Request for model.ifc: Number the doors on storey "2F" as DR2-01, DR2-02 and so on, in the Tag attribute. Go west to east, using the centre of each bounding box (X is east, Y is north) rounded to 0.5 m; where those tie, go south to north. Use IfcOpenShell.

First a look at what the model holds.

```python
import ifcopenshell
import ifcopenshell.util.element
import ifcopenshell.util.placement

model = ifcopenshell.open("model.ifc")
print(model.schema)
storey = next(s for s in model.by_type("IfcBuildingStorey") if s.Name == "2F")
doors = [e for e in ifcopenshell.util.element.get_decomposition(storey) if e.is_a("IfcDoor")]
for e in sorted(doors, key=lambda e: e.id()):
    origin = ifcopenshell.util.placement.get_local_placement(e.ObjectPlacement)[:3, 3]
    print(e.id(), e.Tag, e.Name, origin.round(2) + 0.0, sep=" | ")
```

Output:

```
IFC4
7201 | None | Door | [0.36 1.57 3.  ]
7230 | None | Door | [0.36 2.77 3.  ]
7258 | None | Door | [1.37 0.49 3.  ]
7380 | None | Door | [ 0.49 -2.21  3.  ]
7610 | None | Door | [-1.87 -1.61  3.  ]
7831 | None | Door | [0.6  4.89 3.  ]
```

```python
import ifcopenshell
import ifcopenshell.geom
import ifcopenshell.util.element
import ifcopenshell.util.shape

model = ifcopenshell.open("model.ifc")
settings = ifcopenshell.geom.settings()
settings.set("use-world-coords", True)


def centre(element):
    shape = ifcopenshell.geom.create_shape(settings, element)
    return ifcopenshell.util.shape.get_bbox_centroid(shape.geometry)


storey = next(s for s in model.by_type("IfcBuildingStorey") if s.Name == "2F")
doors = [e for e in ifcopenshell.util.element.get_decomposition(storey) if e.is_a("IfcDoor")]

# Insertion points can sit at a corner or the storey origin, so sort by the geometry (in metres).
centres = {e: centre(e) for e in doors}
doors.sort(key=lambda e: (round(centres[e][0] / 0.5), centres[e][1]))

for i, e in enumerate(doors, start=1):
    number = f"DR2-{i:02d}"
    e.Tag = number
    print(e.id(), number)

model.write("model_v2.ifc")
```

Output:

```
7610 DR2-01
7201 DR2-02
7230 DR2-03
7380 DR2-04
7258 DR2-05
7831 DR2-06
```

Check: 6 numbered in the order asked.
